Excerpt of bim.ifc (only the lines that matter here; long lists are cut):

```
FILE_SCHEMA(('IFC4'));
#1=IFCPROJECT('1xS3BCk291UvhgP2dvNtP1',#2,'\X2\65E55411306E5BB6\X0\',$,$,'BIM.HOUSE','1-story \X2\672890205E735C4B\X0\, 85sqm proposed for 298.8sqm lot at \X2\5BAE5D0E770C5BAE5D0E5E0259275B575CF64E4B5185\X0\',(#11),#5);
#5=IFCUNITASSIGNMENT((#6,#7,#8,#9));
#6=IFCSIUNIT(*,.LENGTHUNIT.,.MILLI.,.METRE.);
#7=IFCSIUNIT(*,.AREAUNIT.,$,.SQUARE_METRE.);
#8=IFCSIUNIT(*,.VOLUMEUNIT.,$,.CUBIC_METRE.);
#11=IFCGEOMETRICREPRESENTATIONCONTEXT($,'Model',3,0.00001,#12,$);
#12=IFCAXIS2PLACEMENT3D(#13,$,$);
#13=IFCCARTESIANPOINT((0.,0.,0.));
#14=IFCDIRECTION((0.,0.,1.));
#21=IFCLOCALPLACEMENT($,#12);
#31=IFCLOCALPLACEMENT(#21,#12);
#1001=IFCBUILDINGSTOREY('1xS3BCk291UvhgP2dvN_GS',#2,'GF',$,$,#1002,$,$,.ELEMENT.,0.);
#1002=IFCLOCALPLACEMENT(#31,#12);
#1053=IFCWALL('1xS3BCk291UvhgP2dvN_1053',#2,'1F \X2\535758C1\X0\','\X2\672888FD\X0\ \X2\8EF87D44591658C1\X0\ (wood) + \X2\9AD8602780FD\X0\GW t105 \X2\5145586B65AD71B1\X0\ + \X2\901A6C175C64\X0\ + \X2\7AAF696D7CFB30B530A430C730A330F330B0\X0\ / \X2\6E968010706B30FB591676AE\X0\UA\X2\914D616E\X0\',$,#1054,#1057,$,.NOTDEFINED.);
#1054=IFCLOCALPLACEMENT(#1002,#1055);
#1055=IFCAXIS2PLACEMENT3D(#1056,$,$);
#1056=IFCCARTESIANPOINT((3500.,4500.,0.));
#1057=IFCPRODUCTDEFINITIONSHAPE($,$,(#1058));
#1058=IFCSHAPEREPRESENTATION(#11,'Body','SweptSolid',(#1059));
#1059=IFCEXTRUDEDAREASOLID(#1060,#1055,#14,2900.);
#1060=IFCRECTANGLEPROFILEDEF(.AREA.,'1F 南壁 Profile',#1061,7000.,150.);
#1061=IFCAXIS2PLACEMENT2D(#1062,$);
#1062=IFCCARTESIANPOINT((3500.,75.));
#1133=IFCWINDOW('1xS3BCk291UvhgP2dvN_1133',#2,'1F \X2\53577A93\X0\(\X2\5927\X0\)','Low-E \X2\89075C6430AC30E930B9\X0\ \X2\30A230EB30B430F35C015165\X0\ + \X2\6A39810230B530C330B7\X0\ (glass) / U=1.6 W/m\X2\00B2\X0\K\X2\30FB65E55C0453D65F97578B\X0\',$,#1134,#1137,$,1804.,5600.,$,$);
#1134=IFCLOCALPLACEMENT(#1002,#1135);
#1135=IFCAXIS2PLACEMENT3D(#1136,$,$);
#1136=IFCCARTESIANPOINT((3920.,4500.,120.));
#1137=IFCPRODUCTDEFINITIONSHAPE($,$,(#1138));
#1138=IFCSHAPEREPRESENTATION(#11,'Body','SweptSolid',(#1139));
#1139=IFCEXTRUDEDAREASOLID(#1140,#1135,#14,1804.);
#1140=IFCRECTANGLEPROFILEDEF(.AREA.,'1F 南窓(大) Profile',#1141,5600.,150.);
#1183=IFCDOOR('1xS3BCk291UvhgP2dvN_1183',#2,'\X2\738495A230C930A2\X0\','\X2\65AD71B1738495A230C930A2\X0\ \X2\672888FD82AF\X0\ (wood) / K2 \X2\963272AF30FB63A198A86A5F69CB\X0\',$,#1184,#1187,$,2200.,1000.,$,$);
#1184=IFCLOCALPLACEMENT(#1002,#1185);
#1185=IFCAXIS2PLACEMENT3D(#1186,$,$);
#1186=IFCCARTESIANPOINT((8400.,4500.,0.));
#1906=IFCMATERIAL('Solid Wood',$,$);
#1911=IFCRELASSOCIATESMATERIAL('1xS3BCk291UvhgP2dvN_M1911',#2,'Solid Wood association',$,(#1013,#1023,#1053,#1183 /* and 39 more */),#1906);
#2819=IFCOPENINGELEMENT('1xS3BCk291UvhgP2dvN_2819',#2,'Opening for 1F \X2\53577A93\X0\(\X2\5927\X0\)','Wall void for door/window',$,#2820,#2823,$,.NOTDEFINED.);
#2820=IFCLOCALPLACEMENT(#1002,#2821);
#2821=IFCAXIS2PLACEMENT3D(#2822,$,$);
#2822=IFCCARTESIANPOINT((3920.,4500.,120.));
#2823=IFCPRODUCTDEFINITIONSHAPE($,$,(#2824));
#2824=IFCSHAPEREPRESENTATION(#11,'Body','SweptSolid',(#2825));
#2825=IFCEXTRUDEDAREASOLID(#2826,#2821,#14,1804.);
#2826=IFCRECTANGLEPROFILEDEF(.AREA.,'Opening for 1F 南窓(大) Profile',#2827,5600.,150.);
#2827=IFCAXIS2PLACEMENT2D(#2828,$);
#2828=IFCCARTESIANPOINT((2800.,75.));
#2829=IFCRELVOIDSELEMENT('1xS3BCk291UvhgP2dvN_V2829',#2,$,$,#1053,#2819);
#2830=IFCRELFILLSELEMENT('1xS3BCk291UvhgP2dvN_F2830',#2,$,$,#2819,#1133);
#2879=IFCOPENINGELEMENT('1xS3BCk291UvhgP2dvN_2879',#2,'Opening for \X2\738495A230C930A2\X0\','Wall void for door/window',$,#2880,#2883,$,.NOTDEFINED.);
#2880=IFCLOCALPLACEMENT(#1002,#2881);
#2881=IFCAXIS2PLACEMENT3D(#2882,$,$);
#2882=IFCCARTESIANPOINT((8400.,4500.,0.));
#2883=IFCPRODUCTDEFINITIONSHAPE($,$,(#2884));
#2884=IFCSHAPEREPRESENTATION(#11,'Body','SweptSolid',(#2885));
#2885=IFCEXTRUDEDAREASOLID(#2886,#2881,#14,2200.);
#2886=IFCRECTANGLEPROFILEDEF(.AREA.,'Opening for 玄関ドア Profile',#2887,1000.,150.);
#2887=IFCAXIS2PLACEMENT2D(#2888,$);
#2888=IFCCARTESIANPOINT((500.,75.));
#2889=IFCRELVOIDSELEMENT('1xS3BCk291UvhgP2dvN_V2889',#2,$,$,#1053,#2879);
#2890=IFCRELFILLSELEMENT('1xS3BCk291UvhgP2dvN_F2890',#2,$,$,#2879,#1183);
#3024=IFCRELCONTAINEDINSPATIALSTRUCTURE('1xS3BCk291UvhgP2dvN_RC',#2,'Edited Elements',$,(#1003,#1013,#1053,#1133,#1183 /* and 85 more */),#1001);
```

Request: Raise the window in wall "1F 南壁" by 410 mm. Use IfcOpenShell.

```python
import numpy as np
import ifcopenshell
import ifcopenshell.api.geometry
import ifcopenshell.util.placement
import ifcopenshell.util.unit

model = ifcopenshell.open("bim.ifc")
unit_scale = ifcopenshell.util.unit.calculate_unit_scale(model)

window = model.by_guid("1xS3BCk291UvhgP2dvN_1133")
opening = window.FillsVoids[0].RelatingOpeningElement
dz = 0.41 / unit_scale

shift = np.array([0.0, 0.0, dz])
# The window is not placed relative to its opening, so move both.
for product in (opening, window):
    matrix = ifcopenshell.util.placement.get_local_placement(product.ObjectPlacement)
    matrix[:3, 3] += shift
    ifcopenshell.api.geometry.edit_object_placement(model, product=product, matrix=matrix, is_si=False)

print(f"moved by {dz * unit_scale:+.3f} m")

model.write("bim_updated.ifc")
```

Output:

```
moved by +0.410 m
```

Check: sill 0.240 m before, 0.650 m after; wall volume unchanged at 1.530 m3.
